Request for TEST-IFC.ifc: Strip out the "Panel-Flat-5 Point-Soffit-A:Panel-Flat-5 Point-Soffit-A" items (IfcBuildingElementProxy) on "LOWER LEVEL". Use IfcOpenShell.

First a look at what the model holds.

```python
import ifcopenshell
import ifcopenshell.util.element

model = ifcopenshell.open("TEST-IFC.ifc")
print(model.schema)
storey = next(s for s in model.by_type("IfcBuildingStorey") if s.Name == "LOWER LEVEL")
proxies = [e for e in ifcopenshell.util.element.get_decomposition(storey) if e.is_a("IfcBuildingElementProxy")]
seen = {}
for e in proxies:
    element_type = ifcopenshell.util.element.get_type(e)
    name = element_type.Name if element_type not in (None, e) else None
    seen[name] = seen.get(name, 0) + 1
for name, count in sorted(seen.items(), key=str):
    print(count, "x", name)
```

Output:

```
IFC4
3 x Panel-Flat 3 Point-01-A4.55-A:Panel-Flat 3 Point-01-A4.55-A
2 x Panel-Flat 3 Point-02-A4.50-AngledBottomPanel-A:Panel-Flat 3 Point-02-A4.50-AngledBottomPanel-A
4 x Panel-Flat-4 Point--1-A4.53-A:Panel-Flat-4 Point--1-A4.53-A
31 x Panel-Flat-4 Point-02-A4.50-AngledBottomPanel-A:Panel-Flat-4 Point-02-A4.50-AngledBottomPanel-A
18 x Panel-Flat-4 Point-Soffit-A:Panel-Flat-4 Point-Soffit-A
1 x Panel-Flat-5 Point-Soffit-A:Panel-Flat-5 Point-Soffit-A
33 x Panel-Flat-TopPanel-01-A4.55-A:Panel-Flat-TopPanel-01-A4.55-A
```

```python
import ifcopenshell
import ifcopenshell.api.root
import ifcopenshell.util.element

model = ifcopenshell.open("TEST-IFC.ifc")

storey = next(s for s in model.by_type("IfcBuildingStorey") if s.Name == "LOWER LEVEL")
proxies = [e for e in ifcopenshell.util.element.get_decomposition(storey) if e.is_a("IfcBuildingElementProxy")]
targets = [e for e in proxies if (t := ifcopenshell.util.element.get_type(e)) not in (None, e) and t.Name == "Panel-Flat-5 Point-Soffit-A:Panel-Flat-5 Point-Soffit-A"]

for e in targets:
    ifcopenshell.api.root.remove_product(model, product=e)
print(len(targets), "removed")

model.write("TEST-IFC_v2.ifc")
```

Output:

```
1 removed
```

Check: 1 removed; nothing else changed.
